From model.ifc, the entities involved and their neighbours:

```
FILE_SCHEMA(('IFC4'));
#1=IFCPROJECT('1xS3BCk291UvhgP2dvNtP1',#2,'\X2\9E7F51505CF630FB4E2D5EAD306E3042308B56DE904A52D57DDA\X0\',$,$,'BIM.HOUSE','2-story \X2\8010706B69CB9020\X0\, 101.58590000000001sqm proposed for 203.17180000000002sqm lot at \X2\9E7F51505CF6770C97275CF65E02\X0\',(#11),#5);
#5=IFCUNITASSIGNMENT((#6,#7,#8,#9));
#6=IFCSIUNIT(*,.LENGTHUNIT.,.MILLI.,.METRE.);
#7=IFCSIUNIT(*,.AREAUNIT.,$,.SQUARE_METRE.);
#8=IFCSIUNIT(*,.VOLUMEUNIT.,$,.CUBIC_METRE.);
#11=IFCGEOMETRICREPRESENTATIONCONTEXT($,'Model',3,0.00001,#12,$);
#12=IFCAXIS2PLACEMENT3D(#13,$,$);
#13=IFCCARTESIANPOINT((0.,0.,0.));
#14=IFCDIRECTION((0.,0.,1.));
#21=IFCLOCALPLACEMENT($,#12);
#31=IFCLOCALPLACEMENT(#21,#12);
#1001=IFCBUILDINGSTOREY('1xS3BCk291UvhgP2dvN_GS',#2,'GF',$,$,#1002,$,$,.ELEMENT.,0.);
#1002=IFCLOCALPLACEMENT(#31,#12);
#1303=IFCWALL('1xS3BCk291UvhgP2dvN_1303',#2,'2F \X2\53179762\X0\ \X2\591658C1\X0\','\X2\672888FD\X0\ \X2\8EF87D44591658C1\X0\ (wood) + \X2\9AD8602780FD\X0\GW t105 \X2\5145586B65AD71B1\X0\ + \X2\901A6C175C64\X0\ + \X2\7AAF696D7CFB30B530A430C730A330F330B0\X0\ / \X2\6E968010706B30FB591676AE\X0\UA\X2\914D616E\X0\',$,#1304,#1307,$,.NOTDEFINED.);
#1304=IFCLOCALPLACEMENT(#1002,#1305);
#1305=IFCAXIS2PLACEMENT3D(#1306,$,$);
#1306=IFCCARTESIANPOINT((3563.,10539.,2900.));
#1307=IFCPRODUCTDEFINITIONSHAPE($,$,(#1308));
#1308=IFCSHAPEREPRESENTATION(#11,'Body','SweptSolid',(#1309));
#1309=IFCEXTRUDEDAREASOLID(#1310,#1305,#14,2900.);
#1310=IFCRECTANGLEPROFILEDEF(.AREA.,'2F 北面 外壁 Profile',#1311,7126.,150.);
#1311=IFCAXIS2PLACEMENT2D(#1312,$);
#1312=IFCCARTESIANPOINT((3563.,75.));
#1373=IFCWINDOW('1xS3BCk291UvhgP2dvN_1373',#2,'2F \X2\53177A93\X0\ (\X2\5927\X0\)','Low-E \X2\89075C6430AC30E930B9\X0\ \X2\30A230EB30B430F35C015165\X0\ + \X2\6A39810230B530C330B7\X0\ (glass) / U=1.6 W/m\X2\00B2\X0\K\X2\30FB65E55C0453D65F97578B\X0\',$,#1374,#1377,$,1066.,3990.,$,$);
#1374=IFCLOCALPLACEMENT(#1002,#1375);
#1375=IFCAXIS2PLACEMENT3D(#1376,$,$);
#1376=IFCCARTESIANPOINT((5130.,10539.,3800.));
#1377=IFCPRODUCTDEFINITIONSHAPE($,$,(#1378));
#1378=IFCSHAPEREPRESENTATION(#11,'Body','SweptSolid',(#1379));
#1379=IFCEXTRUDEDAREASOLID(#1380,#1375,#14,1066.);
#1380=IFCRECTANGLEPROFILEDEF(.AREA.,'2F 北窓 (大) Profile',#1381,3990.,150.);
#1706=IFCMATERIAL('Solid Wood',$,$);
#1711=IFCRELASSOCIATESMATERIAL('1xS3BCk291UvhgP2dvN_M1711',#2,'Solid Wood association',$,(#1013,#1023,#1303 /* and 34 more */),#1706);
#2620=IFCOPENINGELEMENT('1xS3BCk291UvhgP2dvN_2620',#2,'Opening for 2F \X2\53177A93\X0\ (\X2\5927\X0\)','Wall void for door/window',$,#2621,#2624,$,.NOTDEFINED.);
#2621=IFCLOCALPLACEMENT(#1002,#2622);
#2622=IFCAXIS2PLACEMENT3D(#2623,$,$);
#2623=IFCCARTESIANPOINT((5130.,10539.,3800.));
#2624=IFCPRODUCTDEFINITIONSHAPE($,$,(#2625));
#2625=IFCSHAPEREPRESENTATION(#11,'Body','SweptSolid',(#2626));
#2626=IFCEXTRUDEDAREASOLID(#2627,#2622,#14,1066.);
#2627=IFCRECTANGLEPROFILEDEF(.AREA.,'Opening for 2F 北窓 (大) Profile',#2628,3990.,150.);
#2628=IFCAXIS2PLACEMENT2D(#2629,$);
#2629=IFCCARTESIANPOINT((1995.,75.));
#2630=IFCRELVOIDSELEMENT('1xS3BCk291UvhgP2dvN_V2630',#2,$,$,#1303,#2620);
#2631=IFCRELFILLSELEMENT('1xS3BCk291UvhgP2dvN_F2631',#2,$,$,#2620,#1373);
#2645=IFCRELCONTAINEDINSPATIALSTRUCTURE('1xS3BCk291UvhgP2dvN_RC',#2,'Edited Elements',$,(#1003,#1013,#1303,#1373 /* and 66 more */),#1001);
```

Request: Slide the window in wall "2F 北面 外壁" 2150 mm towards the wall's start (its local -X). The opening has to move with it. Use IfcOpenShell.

```python
import ifcopenshell
import ifcopenshell.api.geometry
import ifcopenshell.util.placement
import ifcopenshell.util.unit

model = ifcopenshell.open("model.ifc")
unit_scale = ifcopenshell.util.unit.calculate_unit_scale(model)

window = model.by_id(1373)
opening = window.FillsVoids[0].RelatingOpeningElement
wall = opening.VoidsElements[0].RelatingBuildingElement

wall_matrix = ifcopenshell.util.placement.get_local_placement(wall.ObjectPlacement)
shift = wall_matrix[:3, 0] * -2.15 / unit_scale
before = ifcopenshell.util.placement.get_local_placement(window.ObjectPlacement)[:3, 3].copy()

# The window is not placed relative to its opening, so move both.
for product in (opening, window):
    matrix = ifcopenshell.util.placement.get_local_placement(product.ObjectPlacement)
    matrix[:3, 3] += shift
    ifcopenshell.api.geometry.edit_object_placement(model, product=product, matrix=matrix, is_si=False)

after = ifcopenshell.util.placement.get_local_placement(window.ObjectPlacement)[:3, 3]
print("window moved by", (after - before).round(3) + 0.0)

model.write("model_v2.ifc")
```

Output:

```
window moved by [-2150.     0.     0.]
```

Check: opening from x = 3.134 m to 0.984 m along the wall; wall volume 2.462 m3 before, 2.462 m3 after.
